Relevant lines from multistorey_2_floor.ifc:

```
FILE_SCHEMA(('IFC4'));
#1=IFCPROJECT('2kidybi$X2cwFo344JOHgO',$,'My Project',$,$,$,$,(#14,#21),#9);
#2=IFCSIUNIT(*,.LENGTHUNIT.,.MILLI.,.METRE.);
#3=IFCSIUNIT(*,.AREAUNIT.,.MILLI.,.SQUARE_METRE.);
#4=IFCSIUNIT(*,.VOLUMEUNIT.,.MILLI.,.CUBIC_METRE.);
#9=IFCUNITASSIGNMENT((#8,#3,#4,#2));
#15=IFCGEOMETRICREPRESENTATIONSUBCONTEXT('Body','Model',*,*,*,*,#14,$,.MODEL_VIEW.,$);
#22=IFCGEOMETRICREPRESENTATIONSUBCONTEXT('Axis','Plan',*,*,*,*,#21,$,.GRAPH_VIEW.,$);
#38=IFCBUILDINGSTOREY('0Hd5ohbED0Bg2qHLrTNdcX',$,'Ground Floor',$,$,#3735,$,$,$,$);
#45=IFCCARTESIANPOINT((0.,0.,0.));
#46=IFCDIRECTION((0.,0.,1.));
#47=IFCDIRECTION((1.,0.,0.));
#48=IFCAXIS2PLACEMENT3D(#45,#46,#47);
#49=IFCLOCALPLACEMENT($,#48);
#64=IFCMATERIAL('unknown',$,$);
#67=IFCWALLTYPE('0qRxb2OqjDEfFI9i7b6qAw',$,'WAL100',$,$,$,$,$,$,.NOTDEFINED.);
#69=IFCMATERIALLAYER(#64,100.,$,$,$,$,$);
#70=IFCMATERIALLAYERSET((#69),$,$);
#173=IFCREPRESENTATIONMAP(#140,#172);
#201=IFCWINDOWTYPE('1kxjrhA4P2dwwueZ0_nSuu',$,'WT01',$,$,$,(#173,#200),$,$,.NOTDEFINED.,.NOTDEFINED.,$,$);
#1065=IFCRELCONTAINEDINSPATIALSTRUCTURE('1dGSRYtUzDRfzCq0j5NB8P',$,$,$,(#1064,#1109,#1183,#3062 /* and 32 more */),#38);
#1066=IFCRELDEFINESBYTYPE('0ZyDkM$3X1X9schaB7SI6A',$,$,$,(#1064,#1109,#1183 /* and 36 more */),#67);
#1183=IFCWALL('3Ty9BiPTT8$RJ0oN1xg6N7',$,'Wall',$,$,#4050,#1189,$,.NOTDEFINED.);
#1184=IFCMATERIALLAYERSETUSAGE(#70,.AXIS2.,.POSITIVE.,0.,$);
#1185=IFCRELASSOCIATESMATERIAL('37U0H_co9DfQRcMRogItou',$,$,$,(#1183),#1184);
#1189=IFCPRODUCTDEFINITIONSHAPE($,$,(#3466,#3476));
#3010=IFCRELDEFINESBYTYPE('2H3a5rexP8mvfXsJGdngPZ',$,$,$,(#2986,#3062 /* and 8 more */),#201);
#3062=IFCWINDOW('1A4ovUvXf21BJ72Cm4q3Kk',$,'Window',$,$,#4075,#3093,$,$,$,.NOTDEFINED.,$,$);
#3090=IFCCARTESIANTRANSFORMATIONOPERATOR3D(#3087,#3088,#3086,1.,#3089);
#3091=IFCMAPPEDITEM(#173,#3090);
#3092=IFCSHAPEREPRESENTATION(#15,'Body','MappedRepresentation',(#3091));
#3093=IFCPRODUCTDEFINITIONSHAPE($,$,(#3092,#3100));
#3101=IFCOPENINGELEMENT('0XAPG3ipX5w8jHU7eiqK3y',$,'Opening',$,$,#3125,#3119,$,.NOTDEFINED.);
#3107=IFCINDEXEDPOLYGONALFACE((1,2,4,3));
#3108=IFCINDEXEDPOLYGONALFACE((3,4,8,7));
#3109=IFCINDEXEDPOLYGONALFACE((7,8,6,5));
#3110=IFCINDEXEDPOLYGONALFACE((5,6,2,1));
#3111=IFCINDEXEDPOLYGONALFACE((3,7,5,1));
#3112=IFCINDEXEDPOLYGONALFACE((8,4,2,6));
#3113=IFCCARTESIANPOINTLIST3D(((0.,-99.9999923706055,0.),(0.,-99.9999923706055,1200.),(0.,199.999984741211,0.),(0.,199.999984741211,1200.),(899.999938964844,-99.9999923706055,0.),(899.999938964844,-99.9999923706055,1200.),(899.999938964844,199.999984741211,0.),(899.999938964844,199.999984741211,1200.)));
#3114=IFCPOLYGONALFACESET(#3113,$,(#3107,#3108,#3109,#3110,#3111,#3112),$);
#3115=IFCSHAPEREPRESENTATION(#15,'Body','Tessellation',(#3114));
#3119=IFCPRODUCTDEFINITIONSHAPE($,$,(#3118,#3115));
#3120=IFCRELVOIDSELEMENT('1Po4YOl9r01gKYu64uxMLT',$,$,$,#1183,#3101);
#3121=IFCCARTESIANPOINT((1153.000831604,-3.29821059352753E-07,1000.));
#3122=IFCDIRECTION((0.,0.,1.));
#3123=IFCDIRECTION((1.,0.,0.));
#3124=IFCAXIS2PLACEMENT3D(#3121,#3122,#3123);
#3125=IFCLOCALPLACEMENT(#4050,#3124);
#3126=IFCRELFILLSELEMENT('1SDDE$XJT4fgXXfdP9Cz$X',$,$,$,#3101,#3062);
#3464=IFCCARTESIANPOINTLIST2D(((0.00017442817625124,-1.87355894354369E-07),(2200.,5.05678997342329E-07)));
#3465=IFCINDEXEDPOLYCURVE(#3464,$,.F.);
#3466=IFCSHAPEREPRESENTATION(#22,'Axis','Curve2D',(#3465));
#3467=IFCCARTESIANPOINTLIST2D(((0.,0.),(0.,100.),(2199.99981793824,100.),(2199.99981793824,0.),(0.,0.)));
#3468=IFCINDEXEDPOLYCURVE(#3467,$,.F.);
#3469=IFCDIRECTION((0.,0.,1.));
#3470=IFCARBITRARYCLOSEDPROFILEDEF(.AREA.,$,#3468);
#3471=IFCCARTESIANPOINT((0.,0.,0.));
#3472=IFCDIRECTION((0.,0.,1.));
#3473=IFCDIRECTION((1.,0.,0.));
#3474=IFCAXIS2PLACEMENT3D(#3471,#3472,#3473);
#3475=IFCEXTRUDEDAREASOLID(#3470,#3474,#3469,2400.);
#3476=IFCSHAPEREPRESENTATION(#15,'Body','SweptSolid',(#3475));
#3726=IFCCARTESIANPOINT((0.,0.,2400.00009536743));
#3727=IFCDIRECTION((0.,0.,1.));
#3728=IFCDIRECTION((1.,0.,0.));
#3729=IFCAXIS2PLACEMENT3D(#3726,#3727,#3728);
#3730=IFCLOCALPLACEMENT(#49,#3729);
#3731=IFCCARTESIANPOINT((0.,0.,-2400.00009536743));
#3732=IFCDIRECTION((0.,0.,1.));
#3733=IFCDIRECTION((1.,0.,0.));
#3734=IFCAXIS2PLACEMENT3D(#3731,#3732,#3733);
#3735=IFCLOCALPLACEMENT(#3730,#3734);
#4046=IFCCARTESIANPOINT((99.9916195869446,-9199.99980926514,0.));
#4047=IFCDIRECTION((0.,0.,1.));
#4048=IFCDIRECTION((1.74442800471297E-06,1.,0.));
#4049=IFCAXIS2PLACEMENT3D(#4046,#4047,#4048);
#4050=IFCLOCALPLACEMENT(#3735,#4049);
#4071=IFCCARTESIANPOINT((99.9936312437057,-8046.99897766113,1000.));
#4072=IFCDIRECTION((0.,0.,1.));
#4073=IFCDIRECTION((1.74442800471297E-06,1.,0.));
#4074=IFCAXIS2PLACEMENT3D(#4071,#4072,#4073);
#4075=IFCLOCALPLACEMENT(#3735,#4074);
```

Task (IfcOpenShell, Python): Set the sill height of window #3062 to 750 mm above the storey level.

```python
import numpy as np
import ifcopenshell
import ifcopenshell.api.geometry
import ifcopenshell.geom
import ifcopenshell.util.element
import ifcopenshell.util.placement
import ifcopenshell.util.shape
import ifcopenshell.util.unit

model = ifcopenshell.open("multistorey_2_floor.ifc")
unit_scale = ifcopenshell.util.unit.calculate_unit_scale(model)

window = model.by_id(3062)
opening = window.FillsVoids[0].RelatingOpeningElement
storey = ifcopenshell.util.element.get_container(window, ifc_class="IfcBuildingStorey")
level = ifcopenshell.util.placement.get_local_placement(storey.ObjectPlacement)[2, 3]

# The opening's origin need not be at the sill, so measure its lowest point.
shape = ifcopenshell.geom.create_shape(ifcopenshell.geom.settings(), opening)
bottom = ifcopenshell.util.shape.get_shape_bottom_elevation(shape, shape.geometry) / unit_scale
dz = level + 750.0 - bottom

shift = np.array([0.0, 0.0, dz])
# The window is not placed relative to its opening, so move both.
for product in (opening, window):
    matrix = ifcopenshell.util.placement.get_local_placement(product.ObjectPlacement)
    matrix[:3, 3] += shift
    ifcopenshell.api.geometry.edit_object_placement(model, product=product, matrix=matrix, is_si=False)

print(f"moved by {dz * unit_scale:+.3f} m")

model.write("multistorey_2_floor_rev.ifc")
```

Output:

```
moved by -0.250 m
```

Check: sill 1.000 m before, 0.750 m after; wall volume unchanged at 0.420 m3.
